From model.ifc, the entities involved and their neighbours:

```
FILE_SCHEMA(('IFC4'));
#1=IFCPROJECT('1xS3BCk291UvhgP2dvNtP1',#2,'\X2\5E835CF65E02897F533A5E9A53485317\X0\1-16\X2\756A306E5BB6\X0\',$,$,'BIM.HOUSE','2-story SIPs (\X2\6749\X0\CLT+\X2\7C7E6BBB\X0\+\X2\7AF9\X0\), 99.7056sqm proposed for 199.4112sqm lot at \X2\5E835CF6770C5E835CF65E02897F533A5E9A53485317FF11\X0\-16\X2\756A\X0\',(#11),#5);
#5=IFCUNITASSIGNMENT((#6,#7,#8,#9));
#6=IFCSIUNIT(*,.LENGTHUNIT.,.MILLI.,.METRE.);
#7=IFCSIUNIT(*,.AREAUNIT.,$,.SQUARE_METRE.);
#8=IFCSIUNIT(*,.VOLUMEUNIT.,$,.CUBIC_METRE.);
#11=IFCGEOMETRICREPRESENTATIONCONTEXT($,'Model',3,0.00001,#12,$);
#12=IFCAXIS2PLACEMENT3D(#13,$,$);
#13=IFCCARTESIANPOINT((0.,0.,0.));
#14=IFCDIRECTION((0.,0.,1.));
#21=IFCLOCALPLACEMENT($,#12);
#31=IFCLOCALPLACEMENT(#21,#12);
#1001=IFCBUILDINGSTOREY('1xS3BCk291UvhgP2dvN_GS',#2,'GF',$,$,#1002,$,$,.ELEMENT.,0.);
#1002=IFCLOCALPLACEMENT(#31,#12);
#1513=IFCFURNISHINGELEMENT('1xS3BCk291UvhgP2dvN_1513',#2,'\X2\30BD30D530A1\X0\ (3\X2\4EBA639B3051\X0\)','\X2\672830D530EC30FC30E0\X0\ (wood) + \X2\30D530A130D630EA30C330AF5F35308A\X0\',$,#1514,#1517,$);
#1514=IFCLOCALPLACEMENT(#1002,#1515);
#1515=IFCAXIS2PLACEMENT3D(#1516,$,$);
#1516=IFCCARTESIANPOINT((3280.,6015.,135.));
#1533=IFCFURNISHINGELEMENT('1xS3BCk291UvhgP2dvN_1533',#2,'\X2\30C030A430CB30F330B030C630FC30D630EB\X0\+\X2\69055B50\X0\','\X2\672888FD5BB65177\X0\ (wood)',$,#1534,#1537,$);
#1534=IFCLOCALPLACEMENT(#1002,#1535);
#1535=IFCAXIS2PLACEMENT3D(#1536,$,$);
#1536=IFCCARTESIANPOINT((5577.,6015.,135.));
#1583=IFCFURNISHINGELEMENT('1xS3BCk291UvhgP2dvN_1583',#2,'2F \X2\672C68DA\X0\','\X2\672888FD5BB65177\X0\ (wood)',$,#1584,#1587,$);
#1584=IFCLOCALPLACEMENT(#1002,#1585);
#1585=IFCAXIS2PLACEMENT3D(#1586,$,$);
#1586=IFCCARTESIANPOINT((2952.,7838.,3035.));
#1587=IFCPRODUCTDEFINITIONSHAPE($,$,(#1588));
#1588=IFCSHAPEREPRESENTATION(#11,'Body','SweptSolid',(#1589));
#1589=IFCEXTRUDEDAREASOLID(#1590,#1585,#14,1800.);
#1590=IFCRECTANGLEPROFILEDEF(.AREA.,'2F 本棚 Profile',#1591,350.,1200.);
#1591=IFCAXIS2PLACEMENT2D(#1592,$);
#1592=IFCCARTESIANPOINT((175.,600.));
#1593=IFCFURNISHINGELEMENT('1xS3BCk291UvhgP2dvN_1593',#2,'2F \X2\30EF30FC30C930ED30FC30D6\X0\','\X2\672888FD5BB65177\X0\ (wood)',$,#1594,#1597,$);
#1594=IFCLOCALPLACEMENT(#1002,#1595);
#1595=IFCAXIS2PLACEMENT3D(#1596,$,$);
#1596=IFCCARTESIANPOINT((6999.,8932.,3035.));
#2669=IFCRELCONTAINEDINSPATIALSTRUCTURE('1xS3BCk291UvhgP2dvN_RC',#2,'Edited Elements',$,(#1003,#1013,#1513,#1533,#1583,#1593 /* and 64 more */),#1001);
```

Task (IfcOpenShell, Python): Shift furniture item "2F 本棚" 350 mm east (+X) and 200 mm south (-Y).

```python
import ifcopenshell
import ifcopenshell.api.geometry
import ifcopenshell.util.placement
import ifcopenshell.util.unit

model = ifcopenshell.open("model.ifc")
unit_scale = ifcopenshell.util.unit.calculate_unit_scale(model)

item = model.by_guid("1xS3BCk291UvhgP2dvN_1583")
matrix = ifcopenshell.util.placement.get_local_placement(item.ObjectPlacement)
matrix[0, 3] += 0.35 / unit_scale
matrix[1, 3] -= 0.2 / unit_scale
ifcopenshell.api.geometry.edit_object_placement(model, product=item, matrix=matrix, is_si=False)

print(ifcopenshell.util.placement.get_local_placement(item.ObjectPlacement).round(3) + 0.0)

model.write("model_rev.ifc")
```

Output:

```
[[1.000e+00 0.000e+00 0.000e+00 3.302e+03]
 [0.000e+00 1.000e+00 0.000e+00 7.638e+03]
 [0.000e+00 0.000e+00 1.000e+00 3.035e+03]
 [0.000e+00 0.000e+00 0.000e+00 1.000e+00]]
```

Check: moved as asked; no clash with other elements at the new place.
